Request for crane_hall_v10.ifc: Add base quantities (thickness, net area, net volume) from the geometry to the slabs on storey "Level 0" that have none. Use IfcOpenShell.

First a look at what the model holds.

```python
import ifcopenshell
import ifcopenshell.util.element
import ifcopenshell.util.unit

model = ifcopenshell.open("crane_hall_v10.ifc")
print(model.schema)
for unit_type in ("LENGTHUNIT", "AREAUNIT", "VOLUMEUNIT"):
    print(unit_type, ifcopenshell.util.unit.calculate_unit_scale(model, unit_type))
storey = next(s for s in model.by_type("IfcBuildingStorey") if s.Name == "Level 0")
slabs = [e for e in ifcopenshell.util.element.get_decomposition(storey) if e.is_a("IfcSlab")]
for e in sorted(slabs, key=lambda e: e.id()):
    print(e.id(), e.is_a(), e.Name, list(ifcopenshell.util.element.get_psets(e, qtos_only=True)), sep=" | ")
```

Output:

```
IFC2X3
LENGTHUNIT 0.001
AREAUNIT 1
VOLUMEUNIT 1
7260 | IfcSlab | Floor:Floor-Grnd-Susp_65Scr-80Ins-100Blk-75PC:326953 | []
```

```python
import ifcopenshell
import ifcopenshell.api.pset
import ifcopenshell.geom
import ifcopenshell.util.element
import ifcopenshell.util.shape
import ifcopenshell.util.unit

model = ifcopenshell.open("crane_hall_v10.ifc")
unit_scale = ifcopenshell.util.unit.calculate_unit_scale(model)
area_scale = ifcopenshell.util.unit.calculate_unit_scale(model, "AREAUNIT")
volume_scale = ifcopenshell.util.unit.calculate_unit_scale(model, "VOLUMEUNIT")
settings = ifcopenshell.geom.settings()

storey = next(s for s in model.by_type("IfcBuildingStorey") if s.Name == "Level 0")
slabs = [e for e in ifcopenshell.util.element.get_decomposition(storey) if e.is_a("IfcSlab")]

for e in sorted(slabs, key=lambda e: e.id()):
    if ifcopenshell.util.element.get_psets(e, qtos_only=True, should_inherit=False):
        continue
    # Geometry comes back in metres, in the element's own axes.
    shape = ifcopenshell.geom.create_shape(settings, e)
    values = {
        "Width": ifcopenshell.util.shape.get_z(shape.geometry) / unit_scale,
        "NetArea": ifcopenshell.util.shape.get_footprint_area(shape.geometry) / area_scale,
        "NetVolume": ifcopenshell.util.shape.get_volume(shape.geometry) / volume_scale,
    }
    qto = ifcopenshell.api.pset.add_qto(model, product=e, name="BaseQuantities")
    ifcopenshell.api.pset.edit_qto(model, qto=qto, properties=values)
    print(e.id(), {k: round(v, 3) for k, v in values.items()})

model.write("crane_hall_v10_updated.ifc")
```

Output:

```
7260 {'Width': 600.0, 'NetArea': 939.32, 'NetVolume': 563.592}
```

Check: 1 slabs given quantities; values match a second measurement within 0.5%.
